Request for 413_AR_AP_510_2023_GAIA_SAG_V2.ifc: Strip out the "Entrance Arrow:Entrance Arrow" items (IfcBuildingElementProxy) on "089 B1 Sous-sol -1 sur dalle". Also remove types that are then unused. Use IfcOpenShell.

First a look at what the model holds.

```python
import ifcopenshell
import ifcopenshell.util.element

model = ifcopenshell.open("413_AR_AP_510_2023_GAIA_SAG_V2.ifc")
print(model.schema)
storey = next(s for s in model.by_type("IfcBuildingStorey") if s.Name == "089 B1 Sous-sol -1 sur dalle")
proxies = [e for e in ifcopenshell.util.element.get_decomposition(storey) if e.is_a("IfcBuildingElementProxy")]
seen = {}
for e in proxies:
    element_type = ifcopenshell.util.element.get_type(e)
    name = element_type.Name if element_type not in (None, e) else None
    seen[name] = seen.get(name, 0) + 1
for name, count in sorted(seen.items(), key=str):
    print(count, "x", name)
```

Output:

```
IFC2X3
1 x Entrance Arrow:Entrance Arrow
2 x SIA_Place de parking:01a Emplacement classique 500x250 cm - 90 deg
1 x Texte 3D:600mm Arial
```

```python
import ifcopenshell
import ifcopenshell.api.root
import ifcopenshell.util.element

model = ifcopenshell.open("413_AR_AP_510_2023_GAIA_SAG_V2.ifc")

storey = next(s for s in model.by_type("IfcBuildingStorey") if s.Name == "089 B1 Sous-sol -1 sur dalle")
proxies = [e for e in ifcopenshell.util.element.get_decomposition(storey) if e.is_a("IfcBuildingElementProxy")]
targets = [e for e in proxies if (t := ifcopenshell.util.element.get_type(e)) not in (None, e) and t.Name == "Entrance Arrow:Entrance Arrow"]
types = {ifcopenshell.util.element.get_type(e) for e in targets} - {None, *targets}

for e in targets:
    ifcopenshell.api.root.remove_product(model, product=e)
print(len(targets), "removed")

unused = [t for t in types if not ifcopenshell.util.element.get_types(t)]
for t in unused:
    ifcopenshell.api.root.remove_product(model, product=t)
print(len(unused), "unused types removed")

model.write("413_AR_AP_510_2023_GAIA_SAG_V2_edited.ifc")
```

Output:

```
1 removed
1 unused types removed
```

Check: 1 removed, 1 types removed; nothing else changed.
